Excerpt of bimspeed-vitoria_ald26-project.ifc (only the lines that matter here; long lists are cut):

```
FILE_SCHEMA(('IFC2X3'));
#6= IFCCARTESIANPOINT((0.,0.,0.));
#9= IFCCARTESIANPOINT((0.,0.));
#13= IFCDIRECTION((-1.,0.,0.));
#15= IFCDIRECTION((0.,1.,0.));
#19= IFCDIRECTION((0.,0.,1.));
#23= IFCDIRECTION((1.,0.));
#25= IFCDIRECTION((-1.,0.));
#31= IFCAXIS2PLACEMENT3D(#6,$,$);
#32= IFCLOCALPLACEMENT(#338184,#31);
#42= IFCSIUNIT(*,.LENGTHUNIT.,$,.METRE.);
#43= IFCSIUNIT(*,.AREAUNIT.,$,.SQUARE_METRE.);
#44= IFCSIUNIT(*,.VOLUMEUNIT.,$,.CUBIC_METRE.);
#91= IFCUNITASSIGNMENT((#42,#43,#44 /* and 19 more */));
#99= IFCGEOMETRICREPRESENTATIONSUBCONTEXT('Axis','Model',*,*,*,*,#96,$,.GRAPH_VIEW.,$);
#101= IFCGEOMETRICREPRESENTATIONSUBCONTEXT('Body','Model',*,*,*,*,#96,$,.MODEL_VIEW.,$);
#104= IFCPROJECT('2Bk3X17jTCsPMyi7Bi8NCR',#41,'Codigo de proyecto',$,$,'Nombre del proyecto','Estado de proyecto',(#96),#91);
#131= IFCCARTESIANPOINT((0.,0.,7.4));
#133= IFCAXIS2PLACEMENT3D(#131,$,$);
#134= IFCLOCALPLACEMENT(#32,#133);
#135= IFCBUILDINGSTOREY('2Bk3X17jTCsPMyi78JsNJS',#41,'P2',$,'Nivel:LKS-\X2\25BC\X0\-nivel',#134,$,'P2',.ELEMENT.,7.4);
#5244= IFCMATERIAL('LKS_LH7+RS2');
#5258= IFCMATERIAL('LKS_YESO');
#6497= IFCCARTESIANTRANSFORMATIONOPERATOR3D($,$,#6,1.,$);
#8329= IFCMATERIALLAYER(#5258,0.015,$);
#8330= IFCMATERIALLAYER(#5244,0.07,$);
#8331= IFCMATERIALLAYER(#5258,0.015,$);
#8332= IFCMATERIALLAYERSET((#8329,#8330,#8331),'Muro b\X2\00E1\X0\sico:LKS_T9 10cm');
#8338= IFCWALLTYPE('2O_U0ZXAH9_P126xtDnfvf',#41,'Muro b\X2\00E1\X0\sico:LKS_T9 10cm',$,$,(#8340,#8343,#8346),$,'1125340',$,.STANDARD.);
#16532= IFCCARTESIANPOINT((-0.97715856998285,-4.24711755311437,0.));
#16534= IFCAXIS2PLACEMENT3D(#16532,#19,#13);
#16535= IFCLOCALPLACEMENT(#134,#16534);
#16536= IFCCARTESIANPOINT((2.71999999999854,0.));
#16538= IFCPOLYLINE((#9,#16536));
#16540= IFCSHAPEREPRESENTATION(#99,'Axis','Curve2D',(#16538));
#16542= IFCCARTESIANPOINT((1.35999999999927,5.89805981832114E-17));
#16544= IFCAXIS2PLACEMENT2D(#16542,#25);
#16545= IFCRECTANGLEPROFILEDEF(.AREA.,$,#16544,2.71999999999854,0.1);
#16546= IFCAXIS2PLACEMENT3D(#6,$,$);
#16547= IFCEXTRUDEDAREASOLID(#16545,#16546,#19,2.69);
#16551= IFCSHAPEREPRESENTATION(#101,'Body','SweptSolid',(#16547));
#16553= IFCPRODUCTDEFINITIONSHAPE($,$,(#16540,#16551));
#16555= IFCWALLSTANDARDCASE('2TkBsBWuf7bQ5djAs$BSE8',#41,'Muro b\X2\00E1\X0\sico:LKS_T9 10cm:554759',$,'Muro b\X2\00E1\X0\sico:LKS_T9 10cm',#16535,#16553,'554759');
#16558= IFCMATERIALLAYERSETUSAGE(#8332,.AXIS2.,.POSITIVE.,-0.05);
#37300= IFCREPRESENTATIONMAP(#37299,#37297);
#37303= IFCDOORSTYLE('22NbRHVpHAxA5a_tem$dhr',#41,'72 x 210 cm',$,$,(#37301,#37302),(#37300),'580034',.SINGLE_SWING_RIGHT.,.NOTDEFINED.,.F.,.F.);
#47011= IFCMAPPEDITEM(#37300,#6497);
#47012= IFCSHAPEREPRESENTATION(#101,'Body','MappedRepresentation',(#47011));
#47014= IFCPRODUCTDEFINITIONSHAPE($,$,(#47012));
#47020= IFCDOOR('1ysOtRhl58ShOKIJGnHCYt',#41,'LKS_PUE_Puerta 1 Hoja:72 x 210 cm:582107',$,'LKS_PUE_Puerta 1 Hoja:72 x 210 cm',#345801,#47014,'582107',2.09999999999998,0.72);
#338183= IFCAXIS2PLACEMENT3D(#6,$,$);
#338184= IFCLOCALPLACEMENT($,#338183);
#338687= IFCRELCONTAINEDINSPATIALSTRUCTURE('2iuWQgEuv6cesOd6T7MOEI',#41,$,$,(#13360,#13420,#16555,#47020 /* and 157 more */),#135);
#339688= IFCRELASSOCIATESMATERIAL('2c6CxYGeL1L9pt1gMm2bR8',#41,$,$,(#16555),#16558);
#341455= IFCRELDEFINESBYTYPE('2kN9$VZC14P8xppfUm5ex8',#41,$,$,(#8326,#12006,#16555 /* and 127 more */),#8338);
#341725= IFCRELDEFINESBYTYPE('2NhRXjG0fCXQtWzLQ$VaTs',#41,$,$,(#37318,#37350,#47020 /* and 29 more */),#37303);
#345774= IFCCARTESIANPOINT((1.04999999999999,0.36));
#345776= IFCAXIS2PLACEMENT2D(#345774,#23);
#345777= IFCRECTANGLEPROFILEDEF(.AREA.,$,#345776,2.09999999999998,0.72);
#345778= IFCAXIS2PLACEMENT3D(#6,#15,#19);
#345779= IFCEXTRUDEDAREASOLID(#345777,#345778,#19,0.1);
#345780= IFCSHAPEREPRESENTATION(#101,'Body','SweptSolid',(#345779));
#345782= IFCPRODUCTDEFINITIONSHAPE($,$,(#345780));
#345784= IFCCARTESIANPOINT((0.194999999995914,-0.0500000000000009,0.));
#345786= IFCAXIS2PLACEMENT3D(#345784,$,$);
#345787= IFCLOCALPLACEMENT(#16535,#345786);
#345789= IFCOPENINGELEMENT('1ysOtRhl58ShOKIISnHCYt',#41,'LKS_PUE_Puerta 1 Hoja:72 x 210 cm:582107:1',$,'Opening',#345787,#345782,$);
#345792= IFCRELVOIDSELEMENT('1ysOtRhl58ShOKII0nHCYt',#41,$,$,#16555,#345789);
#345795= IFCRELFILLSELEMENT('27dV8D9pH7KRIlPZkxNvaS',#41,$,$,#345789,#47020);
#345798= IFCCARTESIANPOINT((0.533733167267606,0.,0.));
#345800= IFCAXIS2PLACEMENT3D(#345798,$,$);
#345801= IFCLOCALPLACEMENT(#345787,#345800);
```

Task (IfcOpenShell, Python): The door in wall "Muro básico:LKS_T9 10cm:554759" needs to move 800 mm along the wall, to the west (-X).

```python
import ifcopenshell
import ifcopenshell.api.geometry
import ifcopenshell.util.placement

model = ifcopenshell.open("bimspeed-vitoria_ald26-project.ifc")

door = model.by_id(47020)
opening = door.FillsVoids[0].RelatingOpeningElement
wall = opening.VoidsElements[0].RelatingBuildingElement

wall_matrix = ifcopenshell.util.placement.get_local_placement(wall.ObjectPlacement)
shift = wall_matrix[:3, 0] * 0.8
before = ifcopenshell.util.placement.get_local_placement(door.ObjectPlacement)[:3, 3].copy()

# The door is placed relative to its opening, so it follows when the opening moves.
matrix = ifcopenshell.util.placement.get_local_placement(opening.ObjectPlacement)
matrix[:3, 3] += shift
ifcopenshell.api.geometry.edit_object_placement(
    model, product=opening, matrix=matrix, is_si=False, should_transform_children=True
)

after = ifcopenshell.util.placement.get_local_placement(door.ObjectPlacement)[:3, 3]
print("door moved by", (after - before).round(3) + 0.0)

model.write("bimspeed-vitoria_ald26-project_rev.ifc")
```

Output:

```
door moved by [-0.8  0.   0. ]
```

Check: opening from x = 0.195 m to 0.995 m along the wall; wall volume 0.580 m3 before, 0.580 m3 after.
